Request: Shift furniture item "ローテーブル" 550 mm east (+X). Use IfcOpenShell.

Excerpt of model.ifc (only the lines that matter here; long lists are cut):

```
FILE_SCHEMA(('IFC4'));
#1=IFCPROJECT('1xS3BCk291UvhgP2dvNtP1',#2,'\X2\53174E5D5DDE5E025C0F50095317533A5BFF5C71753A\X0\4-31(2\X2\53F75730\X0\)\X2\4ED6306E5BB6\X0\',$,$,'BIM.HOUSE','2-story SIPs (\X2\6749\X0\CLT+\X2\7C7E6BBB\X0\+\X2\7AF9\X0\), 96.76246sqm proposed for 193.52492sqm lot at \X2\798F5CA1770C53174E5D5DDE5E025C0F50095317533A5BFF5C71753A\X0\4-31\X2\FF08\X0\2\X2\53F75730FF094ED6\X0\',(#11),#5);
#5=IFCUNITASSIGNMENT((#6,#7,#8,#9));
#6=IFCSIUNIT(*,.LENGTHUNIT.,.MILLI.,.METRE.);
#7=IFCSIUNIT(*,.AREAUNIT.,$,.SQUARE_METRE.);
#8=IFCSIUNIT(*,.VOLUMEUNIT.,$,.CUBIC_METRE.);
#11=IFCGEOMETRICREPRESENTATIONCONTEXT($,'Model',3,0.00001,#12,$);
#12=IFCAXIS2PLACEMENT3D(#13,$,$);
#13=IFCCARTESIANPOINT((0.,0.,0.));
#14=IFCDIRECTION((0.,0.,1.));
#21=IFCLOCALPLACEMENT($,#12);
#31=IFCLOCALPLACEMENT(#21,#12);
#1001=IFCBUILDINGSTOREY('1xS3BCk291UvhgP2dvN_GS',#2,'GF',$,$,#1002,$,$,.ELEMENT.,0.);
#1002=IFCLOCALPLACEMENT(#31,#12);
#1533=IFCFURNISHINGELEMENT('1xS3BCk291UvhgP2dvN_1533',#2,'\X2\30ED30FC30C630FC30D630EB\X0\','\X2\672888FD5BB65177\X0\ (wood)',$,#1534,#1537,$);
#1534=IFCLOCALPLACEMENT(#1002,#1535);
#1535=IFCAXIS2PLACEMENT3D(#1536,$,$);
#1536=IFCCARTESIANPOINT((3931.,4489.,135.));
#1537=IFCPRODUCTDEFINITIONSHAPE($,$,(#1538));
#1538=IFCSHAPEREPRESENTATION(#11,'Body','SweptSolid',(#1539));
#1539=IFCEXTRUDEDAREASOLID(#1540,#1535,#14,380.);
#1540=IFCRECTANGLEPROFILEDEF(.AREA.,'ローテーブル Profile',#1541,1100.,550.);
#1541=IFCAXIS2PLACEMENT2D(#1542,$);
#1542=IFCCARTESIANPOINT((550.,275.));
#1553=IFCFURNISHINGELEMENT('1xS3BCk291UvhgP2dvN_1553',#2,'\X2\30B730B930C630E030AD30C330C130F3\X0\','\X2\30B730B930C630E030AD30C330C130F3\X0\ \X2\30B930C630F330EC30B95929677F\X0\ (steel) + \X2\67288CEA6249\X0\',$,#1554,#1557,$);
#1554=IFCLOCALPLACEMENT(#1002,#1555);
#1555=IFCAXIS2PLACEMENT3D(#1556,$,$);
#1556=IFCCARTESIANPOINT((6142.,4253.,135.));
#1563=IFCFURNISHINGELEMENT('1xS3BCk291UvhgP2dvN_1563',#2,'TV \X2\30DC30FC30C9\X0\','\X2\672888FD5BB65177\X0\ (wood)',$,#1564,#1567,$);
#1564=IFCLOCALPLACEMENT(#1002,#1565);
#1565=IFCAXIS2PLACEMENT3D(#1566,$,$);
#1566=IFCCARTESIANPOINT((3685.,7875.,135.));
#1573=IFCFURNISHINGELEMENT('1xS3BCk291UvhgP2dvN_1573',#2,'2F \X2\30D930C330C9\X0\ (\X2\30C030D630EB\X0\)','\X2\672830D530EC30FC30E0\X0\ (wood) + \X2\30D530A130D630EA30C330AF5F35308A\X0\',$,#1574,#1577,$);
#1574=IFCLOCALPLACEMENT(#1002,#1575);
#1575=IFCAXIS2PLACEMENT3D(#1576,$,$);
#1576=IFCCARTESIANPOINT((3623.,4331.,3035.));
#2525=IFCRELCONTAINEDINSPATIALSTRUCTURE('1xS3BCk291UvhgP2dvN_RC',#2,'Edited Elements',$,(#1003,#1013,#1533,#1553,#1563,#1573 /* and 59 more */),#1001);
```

```python
import ifcopenshell
import ifcopenshell.api.geometry
import ifcopenshell.util.placement

model = ifcopenshell.open("model.ifc")

item = model.by_guid("1xS3BCk291UvhgP2dvN_1533")
matrix = ifcopenshell.util.placement.get_local_placement(item.ObjectPlacement)
matrix[0, 3] += 550.0
ifcopenshell.api.geometry.edit_object_placement(model, product=item, matrix=matrix, is_si=False)

print(ifcopenshell.util.placement.get_local_placement(item.ObjectPlacement).round(3) + 0.0)

model.write("model_rev.ifc")
```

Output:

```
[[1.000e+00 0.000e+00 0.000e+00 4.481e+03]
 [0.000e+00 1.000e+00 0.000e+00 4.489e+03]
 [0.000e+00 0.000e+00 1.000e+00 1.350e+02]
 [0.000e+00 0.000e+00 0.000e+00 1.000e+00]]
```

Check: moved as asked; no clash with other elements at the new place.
